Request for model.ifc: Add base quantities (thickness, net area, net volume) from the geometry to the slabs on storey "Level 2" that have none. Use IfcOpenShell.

First a look at what the model holds.

```python
import ifcopenshell
import ifcopenshell.util.element
import ifcopenshell.util.unit

model = ifcopenshell.open("model.ifc")
print(model.schema)
for unit_type in ("LENGTHUNIT", "AREAUNIT", "VOLUMEUNIT"):
    print(unit_type, ifcopenshell.util.unit.calculate_unit_scale(model, unit_type))
storey = next(s for s in model.by_type("IfcBuildingStorey") if s.Name == "Level 2")
slabs = [e for e in ifcopenshell.util.element.get_decomposition(storey) if e.is_a("IfcSlab")]
for e in sorted(slabs, key=lambda e: e.id()):
    print(e.id(), e.is_a(), e.Name, list(ifcopenshell.util.element.get_psets(e, qtos_only=True)), sep=" | ")
```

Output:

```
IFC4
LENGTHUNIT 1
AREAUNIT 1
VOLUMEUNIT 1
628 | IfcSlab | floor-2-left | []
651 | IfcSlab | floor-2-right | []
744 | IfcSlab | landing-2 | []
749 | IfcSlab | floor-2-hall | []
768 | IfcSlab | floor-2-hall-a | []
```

```python
import ifcopenshell
import ifcopenshell.api.pset
import ifcopenshell.geom
import ifcopenshell.util.element
import ifcopenshell.util.shape
import ifcopenshell.util.unit

model = ifcopenshell.open("model.ifc")
unit_scale = ifcopenshell.util.unit.calculate_unit_scale(model)
area_scale = ifcopenshell.util.unit.calculate_unit_scale(model, "AREAUNIT")
volume_scale = ifcopenshell.util.unit.calculate_unit_scale(model, "VOLUMEUNIT")
settings = ifcopenshell.geom.settings()

storey = next(s for s in model.by_type("IfcBuildingStorey") if s.Name == "Level 2")
slabs = [e for e in ifcopenshell.util.element.get_decomposition(storey) if e.is_a("IfcSlab")]

for e in sorted(slabs, key=lambda e: e.id()):
    if ifcopenshell.util.element.get_psets(e, qtos_only=True, should_inherit=False):
        continue
    # Geometry comes back in metres, in the element's own axes.
    shape = ifcopenshell.geom.create_shape(settings, e)
    values = {
        "Width": ifcopenshell.util.shape.get_z(shape.geometry) / unit_scale,
        "NetArea": ifcopenshell.util.shape.get_footprint_area(shape.geometry) / area_scale,
        "NetVolume": ifcopenshell.util.shape.get_volume(shape.geometry) / volume_scale,
    }
    qto = ifcopenshell.api.pset.add_qto(model, product=e, name="Qto_SlabBaseQuantities")
    ifcopenshell.api.pset.edit_qto(model, qto=qto, properties=values)
    print(e.id(), {k: round(v, 3) for k, v in values.items()})

model.write("model-out.ifc")
```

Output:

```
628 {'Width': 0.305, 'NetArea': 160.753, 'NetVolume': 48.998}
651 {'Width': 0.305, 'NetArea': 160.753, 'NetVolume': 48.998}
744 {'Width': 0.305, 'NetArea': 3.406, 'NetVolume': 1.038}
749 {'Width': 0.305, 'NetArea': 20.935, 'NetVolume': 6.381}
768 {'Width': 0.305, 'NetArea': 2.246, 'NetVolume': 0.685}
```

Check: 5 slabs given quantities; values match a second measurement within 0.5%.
